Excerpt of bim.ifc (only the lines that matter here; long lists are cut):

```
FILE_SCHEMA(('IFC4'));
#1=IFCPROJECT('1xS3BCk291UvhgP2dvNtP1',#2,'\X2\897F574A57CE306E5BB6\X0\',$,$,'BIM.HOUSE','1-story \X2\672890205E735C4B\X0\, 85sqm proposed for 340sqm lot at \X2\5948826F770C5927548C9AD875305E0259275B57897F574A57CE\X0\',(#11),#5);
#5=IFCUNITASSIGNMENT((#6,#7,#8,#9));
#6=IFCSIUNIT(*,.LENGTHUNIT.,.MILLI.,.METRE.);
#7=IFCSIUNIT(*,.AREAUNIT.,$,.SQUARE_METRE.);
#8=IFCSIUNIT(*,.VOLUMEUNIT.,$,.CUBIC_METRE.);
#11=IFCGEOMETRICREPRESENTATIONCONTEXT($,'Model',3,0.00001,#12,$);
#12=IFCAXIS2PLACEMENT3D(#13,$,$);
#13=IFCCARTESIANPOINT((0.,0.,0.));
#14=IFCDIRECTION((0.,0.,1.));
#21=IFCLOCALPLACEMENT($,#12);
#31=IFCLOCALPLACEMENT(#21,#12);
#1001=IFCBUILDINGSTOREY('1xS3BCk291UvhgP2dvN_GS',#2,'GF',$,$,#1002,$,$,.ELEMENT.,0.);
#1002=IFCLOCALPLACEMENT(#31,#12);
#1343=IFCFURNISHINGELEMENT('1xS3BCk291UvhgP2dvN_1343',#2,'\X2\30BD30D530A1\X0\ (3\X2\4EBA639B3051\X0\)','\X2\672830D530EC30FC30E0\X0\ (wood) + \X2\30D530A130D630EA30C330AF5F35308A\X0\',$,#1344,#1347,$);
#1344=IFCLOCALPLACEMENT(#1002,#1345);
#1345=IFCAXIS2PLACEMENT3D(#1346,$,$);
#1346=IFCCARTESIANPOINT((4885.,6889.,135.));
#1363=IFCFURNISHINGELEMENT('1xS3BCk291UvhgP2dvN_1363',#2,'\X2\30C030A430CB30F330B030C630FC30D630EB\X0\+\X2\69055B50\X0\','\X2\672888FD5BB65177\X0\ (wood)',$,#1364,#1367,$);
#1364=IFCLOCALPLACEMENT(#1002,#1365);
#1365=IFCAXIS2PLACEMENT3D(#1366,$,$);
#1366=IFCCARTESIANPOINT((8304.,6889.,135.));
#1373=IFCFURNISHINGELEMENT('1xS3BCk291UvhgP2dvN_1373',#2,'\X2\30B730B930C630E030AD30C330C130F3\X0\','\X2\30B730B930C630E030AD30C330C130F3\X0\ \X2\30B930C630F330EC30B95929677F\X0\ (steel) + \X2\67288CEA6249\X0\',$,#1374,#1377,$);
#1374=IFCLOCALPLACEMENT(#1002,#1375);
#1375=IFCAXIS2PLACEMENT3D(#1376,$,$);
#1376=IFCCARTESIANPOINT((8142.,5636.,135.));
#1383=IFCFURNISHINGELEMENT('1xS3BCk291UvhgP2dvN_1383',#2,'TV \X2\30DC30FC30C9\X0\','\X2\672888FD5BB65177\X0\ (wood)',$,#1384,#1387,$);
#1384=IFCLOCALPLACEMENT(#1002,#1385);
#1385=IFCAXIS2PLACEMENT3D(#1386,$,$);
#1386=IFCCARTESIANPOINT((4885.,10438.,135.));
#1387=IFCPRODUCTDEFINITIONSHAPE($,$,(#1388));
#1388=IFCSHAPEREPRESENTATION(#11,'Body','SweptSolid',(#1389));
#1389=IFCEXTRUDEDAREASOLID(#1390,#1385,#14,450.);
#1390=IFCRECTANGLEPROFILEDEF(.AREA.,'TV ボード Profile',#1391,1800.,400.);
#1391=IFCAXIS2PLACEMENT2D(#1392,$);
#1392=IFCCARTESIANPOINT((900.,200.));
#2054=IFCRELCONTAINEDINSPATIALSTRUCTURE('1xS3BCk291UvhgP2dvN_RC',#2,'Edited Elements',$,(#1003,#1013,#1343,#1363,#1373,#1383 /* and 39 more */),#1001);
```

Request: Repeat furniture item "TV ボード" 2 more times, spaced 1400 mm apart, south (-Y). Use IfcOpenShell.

```python
import numpy as np
import ifcopenshell
import ifcopenshell.api.geometry
import ifcopenshell.api.root
import ifcopenshell.util.element
import ifcopenshell.util.placement

model = ifcopenshell.open("bim.ifc")


def reuse_history(source, copy):
    """copy_class also copies each property set's owner history, people and application; keep the originals."""
    for rel in copy.IsDefinedBy:
        if rel.is_a("IfcRelDefinesByProperties") and (history := rel.RelatingPropertyDefinition.OwnerHistory):
            rel.RelatingPropertyDefinition.OwnerHistory = source.OwnerHistory
            ifcopenshell.util.element.remove_deep2(model, history)


source = model.by_guid("1xS3BCk291UvhgP2dvN_1383")
base = ifcopenshell.util.placement.get_local_placement(source.ObjectPlacement)
step = np.array([0.0, -1.0, 0.0]) * 1400.0

for i in range(1, 3):
    copy = ifcopenshell.api.root.copy_class(model, product=source)
    copy.Representation = ifcopenshell.util.element.copy_deep(
        model, source.Representation, exclude=["IfcGeometricRepresentationContext", "IfcRepresentationMap"]
    )
    reuse_history(source, copy)
    matrix = base.copy()
    matrix[:3, 3] += i * step
    print("added at", matrix[:3, 3].round(3) + 0.0)
    ifcopenshell.api.geometry.edit_object_placement(model, product=copy, matrix=matrix, is_si=False)

model.write("bim_v2.ifc")
```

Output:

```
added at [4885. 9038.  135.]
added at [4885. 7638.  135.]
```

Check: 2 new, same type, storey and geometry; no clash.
